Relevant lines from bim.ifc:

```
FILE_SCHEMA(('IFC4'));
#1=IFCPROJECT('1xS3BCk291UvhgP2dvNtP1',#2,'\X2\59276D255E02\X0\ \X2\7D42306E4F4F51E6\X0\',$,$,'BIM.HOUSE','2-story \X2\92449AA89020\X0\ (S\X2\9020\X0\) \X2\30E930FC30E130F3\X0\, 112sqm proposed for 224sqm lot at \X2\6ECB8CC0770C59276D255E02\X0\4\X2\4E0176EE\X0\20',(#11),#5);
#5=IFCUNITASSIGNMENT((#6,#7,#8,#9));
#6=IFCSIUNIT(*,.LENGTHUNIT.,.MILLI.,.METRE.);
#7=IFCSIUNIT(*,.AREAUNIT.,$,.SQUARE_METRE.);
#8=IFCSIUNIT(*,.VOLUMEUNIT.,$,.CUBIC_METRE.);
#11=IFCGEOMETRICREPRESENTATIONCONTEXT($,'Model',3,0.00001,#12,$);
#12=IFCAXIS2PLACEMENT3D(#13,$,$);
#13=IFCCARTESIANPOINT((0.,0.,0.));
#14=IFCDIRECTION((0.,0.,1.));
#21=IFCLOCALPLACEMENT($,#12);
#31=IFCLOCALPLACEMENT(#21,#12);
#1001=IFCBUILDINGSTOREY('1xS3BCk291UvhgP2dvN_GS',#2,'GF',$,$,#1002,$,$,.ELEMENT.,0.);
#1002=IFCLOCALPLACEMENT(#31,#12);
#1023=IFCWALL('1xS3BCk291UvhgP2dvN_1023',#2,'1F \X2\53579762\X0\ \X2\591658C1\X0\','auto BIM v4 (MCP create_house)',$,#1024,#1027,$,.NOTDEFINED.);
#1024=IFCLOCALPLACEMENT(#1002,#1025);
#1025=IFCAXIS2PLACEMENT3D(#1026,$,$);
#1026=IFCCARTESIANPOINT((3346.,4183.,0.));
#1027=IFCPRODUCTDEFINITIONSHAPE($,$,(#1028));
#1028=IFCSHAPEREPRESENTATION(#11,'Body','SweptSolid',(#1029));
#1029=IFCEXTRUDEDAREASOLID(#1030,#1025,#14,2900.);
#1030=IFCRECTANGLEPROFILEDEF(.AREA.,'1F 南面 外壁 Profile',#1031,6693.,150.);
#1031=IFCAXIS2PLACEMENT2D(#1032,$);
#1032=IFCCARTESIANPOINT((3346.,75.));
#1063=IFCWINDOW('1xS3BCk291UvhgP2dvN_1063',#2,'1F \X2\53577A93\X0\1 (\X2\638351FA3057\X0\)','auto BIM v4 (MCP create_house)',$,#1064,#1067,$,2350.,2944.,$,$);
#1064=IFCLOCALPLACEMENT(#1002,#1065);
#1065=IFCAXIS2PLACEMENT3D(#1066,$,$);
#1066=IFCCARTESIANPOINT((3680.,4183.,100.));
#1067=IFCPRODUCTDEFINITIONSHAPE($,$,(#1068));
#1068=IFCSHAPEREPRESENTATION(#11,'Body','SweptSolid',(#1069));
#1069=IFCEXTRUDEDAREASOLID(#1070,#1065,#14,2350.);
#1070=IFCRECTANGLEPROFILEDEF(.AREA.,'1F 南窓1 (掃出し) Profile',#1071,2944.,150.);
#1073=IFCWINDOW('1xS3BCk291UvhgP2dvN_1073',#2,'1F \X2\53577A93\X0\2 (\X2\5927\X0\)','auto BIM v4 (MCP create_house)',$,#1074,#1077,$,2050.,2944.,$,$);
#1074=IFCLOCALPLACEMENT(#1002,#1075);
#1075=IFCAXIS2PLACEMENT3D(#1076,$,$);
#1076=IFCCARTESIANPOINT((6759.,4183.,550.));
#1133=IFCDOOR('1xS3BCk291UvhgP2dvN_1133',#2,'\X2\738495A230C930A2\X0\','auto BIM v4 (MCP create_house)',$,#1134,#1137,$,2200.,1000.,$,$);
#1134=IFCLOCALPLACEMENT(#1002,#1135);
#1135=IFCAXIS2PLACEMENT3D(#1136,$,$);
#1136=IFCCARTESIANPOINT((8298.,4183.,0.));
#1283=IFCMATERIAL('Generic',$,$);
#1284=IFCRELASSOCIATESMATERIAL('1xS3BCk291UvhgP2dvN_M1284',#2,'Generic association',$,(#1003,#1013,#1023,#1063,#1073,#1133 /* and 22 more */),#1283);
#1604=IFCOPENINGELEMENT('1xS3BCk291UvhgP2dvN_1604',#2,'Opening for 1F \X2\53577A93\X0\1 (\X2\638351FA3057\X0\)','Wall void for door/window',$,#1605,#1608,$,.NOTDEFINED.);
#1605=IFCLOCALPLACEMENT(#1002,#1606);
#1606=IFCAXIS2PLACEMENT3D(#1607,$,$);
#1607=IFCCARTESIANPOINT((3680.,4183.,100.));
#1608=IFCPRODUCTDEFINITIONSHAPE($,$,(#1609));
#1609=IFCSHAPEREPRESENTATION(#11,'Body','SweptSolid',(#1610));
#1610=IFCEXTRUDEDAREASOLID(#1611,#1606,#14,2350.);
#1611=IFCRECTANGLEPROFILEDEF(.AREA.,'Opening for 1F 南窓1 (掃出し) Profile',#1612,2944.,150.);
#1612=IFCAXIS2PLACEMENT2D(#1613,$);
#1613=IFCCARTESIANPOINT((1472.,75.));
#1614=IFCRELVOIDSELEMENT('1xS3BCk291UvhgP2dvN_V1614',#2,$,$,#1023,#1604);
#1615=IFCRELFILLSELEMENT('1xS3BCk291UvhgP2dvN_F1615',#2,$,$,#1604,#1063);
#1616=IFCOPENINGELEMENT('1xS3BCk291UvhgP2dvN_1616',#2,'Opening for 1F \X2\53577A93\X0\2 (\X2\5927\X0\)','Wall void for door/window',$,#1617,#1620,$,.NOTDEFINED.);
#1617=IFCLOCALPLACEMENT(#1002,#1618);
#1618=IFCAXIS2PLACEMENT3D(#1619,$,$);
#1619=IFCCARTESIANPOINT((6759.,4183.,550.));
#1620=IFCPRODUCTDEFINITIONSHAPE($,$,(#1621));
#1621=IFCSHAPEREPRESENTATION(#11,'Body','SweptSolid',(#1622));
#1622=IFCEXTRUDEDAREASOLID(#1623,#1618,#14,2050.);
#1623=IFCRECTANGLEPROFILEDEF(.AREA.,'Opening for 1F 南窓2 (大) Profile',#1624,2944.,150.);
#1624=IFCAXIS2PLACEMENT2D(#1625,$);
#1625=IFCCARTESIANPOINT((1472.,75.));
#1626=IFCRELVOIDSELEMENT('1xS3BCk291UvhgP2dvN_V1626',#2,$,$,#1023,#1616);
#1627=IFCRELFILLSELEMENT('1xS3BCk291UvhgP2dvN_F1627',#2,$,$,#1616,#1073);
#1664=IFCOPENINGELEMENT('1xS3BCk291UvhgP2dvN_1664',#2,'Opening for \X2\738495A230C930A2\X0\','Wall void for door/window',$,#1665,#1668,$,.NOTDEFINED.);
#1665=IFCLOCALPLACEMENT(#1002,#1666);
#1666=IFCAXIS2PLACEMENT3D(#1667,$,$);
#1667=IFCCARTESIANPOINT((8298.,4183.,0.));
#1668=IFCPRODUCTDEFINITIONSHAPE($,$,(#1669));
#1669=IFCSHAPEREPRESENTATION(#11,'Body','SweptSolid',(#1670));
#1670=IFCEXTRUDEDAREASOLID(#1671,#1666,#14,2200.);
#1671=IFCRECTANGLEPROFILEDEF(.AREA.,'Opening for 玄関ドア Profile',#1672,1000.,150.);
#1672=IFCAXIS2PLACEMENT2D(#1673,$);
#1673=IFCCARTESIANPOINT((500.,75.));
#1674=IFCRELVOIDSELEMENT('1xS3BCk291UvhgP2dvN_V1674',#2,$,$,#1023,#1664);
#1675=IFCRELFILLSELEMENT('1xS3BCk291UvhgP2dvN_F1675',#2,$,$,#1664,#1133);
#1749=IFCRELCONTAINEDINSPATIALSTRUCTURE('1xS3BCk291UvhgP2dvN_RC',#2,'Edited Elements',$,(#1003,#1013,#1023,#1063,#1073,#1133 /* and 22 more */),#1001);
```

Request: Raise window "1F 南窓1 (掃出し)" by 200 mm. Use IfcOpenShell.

```python
import numpy as np
import ifcopenshell
import ifcopenshell.api.geometry
import ifcopenshell.util.placement
import ifcopenshell.util.unit

model = ifcopenshell.open("bim.ifc")
unit_scale = ifcopenshell.util.unit.calculate_unit_scale(model)

window = model.by_guid("1xS3BCk291UvhgP2dvN_1063")
opening = window.FillsVoids[0].RelatingOpeningElement
dz = 0.2 / unit_scale

shift = np.array([0.0, 0.0, dz])
# The window is not placed relative to its opening, so move both.
for product in (opening, window):
    matrix = ifcopenshell.util.placement.get_local_placement(product.ObjectPlacement)
    matrix[:3, 3] += shift
    ifcopenshell.api.geometry.edit_object_placement(model, product=product, matrix=matrix, is_si=False)

print(f"moved by {dz * unit_scale:+.3f} m")

model.write("bim_v2.ifc")
```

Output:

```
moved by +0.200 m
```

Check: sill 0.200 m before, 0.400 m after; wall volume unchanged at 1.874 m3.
